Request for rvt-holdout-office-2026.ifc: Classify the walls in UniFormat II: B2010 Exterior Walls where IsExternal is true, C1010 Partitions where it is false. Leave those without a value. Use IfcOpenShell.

First a look at what the model holds.

```python
import ifcopenshell
import ifcopenshell.util.element

model = ifcopenshell.open("rvt-holdout-office-2026.ifc")
print(model.schema)
print("classifications:", [c.Name for c in model.by_type("IfcClassification")])
values = [ifcopenshell.util.element.get_pset(e, "Pset_WallCommon", "IsExternal") for e in model.by_type("IfcWall")]
for value in (True, False, None):
    print("IsExternal", value, values.count(value))
```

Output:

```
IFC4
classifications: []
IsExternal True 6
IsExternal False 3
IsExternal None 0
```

```python
import ifcopenshell
import ifcopenshell.api.classification
import ifcopenshell.util.element

model = ifcopenshell.open("rvt-holdout-office-2026.ifc")

system = ifcopenshell.api.classification.add_classification(model, classification="UniFormat II")

walls = model.by_type("IfcWall")
external = {e: ifcopenshell.util.element.get_pset(e, "Pset_WallCommon", "IsExternal") for e in walls}
for flag, code, name in ((True, "B2010", "Exterior Walls"), (False, "C1010", "Partitions")):
    products = [e for e in walls if external[e] is flag]
    ifcopenshell.api.classification.add_reference(
        model, products=products, classification=system, identification=code, name=name
    )
    print(code, len(products))

model.write("rvt-holdout-office-2026-out.ifc")
```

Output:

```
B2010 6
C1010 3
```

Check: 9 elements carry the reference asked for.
